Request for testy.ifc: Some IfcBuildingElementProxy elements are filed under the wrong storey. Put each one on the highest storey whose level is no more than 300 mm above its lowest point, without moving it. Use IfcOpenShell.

First a look at what the model holds.

```python
import ifcopenshell
import ifcopenshell.util.element
import ifcopenshell.util.placement

model = ifcopenshell.open("testy.ifc")
print(model.schema)
for storey in model.by_type("IfcBuildingStorey"):
    level = ifcopenshell.util.placement.get_storey_elevation(storey)
    count = sum(e.is_a("IfcBuildingElementProxy") for e in ifcopenshell.util.element.get_contained(storey))
    print(storey.id(), storey.Name, round(level, 3), count, sep=" | ")
```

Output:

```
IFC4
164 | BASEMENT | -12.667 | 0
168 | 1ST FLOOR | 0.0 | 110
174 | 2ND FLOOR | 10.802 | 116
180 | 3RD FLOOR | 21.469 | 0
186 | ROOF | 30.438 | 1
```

```python
import ifcopenshell
import ifcopenshell.api.spatial
import ifcopenshell.geom
import ifcopenshell.util.element
import ifcopenshell.util.placement
import ifcopenshell.util.shape
import ifcopenshell.util.unit

model = ifcopenshell.open("testy.ifc")
unit_scale = ifcopenshell.util.unit.calculate_unit_scale(model)
settings = ifcopenshell.geom.settings()

levels = sorted(
    ((ifcopenshell.util.placement.get_storey_elevation(s) * unit_scale, s) for s in model.by_type("IfcBuildingStorey")),
    key=lambda pair: pair[0],
)

for e in model.by_type("IfcBuildingElementProxy"):
    current = e.ContainedInStructure[0].RelatingStructure if e.ContainedInStructure else None
    if current is None or not current.is_a("IfcBuildingStorey"):
        continue
    shape = ifcopenshell.geom.create_shape(settings, e)
    bottom = ifcopenshell.util.shape.get_shape_bottom_elevation(shape, shape.geometry)
    below = [s for level, s in levels if level <= bottom + 0.3]
    storey = below[-1] if below else levels[0][1]
    if storey != current:
        # assign_container keeps the world position.
        ifcopenshell.api.spatial.assign_container(model, products=[e], relating_structure=storey)
        print(e.id(), current.Name, "->", storey.Name)

model.write("testy_updated.ifc")
```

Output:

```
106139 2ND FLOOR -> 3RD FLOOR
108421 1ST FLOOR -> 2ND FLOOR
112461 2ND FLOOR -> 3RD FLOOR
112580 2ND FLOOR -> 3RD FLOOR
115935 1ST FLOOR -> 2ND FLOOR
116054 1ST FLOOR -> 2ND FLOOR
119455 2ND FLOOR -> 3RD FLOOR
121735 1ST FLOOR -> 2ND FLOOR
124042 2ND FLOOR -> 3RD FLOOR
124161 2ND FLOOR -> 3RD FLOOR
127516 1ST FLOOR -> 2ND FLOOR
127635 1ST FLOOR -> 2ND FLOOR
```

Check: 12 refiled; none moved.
